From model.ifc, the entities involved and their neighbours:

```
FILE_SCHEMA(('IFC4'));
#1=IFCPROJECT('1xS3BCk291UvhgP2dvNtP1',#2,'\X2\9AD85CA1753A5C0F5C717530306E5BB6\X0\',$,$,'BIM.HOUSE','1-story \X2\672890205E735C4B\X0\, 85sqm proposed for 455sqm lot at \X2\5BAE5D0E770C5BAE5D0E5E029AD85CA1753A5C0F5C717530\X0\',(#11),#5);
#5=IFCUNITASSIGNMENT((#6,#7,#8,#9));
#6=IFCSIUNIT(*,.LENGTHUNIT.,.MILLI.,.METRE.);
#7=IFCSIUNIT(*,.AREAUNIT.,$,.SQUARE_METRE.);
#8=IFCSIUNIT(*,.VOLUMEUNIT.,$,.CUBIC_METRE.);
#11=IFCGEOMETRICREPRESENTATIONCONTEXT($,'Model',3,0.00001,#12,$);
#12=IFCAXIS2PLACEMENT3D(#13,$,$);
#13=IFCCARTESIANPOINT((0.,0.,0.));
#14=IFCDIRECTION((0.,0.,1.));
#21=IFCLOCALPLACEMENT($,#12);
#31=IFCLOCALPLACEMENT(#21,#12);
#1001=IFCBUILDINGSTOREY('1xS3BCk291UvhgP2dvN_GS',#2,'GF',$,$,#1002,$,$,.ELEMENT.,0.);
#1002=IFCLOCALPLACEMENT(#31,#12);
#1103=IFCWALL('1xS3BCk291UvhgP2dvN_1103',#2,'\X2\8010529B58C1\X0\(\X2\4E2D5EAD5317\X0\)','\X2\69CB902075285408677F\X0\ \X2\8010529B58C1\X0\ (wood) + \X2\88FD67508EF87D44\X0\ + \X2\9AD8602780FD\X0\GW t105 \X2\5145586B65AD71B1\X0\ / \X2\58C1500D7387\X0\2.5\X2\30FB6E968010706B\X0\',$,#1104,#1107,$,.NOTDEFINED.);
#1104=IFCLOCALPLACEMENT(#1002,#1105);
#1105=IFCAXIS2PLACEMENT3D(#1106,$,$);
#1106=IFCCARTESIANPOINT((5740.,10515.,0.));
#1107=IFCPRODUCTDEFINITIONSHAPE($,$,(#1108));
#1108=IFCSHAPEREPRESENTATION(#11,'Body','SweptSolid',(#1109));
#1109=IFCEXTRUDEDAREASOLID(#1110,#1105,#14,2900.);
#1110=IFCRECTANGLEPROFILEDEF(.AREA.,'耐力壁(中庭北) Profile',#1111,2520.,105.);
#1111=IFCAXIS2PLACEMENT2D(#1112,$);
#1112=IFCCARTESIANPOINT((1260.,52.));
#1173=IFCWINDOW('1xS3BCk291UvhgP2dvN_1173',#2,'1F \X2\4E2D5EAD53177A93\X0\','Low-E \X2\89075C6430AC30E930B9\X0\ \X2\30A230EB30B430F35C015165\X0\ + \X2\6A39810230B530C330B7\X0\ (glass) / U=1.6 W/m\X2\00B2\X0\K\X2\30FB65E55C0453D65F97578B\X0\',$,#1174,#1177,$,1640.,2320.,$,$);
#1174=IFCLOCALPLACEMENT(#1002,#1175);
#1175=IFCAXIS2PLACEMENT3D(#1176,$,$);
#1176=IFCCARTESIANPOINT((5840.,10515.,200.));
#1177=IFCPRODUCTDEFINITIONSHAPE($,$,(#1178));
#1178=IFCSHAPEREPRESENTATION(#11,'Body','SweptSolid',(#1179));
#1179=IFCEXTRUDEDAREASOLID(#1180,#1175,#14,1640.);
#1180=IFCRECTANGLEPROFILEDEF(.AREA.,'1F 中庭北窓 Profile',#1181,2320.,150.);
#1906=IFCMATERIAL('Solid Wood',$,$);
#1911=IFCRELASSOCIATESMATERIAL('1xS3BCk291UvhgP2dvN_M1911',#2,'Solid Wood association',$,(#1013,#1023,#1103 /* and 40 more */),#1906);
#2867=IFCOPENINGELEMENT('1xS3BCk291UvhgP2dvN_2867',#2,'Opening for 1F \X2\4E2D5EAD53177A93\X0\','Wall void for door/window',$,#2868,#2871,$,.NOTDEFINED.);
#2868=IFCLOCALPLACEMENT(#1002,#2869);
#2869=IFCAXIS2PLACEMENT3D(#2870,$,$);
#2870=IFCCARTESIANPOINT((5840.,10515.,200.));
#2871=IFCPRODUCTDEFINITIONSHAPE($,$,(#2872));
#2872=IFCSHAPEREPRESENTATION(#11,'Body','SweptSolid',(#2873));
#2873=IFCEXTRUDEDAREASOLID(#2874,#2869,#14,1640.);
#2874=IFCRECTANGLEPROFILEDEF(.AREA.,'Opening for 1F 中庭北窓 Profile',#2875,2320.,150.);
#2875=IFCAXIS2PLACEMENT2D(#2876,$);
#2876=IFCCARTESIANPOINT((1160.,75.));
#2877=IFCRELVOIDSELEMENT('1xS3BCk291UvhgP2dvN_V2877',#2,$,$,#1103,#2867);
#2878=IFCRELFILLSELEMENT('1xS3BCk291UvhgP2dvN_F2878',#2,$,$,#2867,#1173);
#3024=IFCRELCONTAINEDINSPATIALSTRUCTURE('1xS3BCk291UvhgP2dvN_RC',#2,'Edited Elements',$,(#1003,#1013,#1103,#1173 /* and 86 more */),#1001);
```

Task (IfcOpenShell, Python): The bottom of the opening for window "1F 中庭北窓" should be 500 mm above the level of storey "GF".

```python
import numpy as np
import ifcopenshell
import ifcopenshell.api.geometry
import ifcopenshell.geom
import ifcopenshell.util.element
import ifcopenshell.util.placement
import ifcopenshell.util.shape
import ifcopenshell.util.unit

model = ifcopenshell.open("model.ifc")
unit_scale = ifcopenshell.util.unit.calculate_unit_scale(model)

window = model.by_guid("1xS3BCk291UvhgP2dvN_1173")
opening = window.FillsVoids[0].RelatingOpeningElement
storey = ifcopenshell.util.element.get_container(window, ifc_class="IfcBuildingStorey")
level = ifcopenshell.util.placement.get_local_placement(storey.ObjectPlacement)[2, 3]

# The opening's origin need not be at the sill, so measure its lowest point.
shape = ifcopenshell.geom.create_shape(ifcopenshell.geom.settings(), opening)
bottom = ifcopenshell.util.shape.get_shape_bottom_elevation(shape, shape.geometry) / unit_scale
dz = level + 500.0 - bottom

shift = np.array([0.0, 0.0, dz])
# The window is not placed relative to its opening, so move both.
for product in (opening, window):
    matrix = ifcopenshell.util.placement.get_local_placement(product.ObjectPlacement)
    matrix[:3, 3] += shift
    ifcopenshell.api.geometry.edit_object_placement(model, product=product, matrix=matrix, is_si=False)

print(f"moved by {dz * unit_scale:+.3f} m")

model.write("model_updated.ifc")
```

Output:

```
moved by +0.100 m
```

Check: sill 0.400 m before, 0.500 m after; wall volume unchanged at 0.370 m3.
